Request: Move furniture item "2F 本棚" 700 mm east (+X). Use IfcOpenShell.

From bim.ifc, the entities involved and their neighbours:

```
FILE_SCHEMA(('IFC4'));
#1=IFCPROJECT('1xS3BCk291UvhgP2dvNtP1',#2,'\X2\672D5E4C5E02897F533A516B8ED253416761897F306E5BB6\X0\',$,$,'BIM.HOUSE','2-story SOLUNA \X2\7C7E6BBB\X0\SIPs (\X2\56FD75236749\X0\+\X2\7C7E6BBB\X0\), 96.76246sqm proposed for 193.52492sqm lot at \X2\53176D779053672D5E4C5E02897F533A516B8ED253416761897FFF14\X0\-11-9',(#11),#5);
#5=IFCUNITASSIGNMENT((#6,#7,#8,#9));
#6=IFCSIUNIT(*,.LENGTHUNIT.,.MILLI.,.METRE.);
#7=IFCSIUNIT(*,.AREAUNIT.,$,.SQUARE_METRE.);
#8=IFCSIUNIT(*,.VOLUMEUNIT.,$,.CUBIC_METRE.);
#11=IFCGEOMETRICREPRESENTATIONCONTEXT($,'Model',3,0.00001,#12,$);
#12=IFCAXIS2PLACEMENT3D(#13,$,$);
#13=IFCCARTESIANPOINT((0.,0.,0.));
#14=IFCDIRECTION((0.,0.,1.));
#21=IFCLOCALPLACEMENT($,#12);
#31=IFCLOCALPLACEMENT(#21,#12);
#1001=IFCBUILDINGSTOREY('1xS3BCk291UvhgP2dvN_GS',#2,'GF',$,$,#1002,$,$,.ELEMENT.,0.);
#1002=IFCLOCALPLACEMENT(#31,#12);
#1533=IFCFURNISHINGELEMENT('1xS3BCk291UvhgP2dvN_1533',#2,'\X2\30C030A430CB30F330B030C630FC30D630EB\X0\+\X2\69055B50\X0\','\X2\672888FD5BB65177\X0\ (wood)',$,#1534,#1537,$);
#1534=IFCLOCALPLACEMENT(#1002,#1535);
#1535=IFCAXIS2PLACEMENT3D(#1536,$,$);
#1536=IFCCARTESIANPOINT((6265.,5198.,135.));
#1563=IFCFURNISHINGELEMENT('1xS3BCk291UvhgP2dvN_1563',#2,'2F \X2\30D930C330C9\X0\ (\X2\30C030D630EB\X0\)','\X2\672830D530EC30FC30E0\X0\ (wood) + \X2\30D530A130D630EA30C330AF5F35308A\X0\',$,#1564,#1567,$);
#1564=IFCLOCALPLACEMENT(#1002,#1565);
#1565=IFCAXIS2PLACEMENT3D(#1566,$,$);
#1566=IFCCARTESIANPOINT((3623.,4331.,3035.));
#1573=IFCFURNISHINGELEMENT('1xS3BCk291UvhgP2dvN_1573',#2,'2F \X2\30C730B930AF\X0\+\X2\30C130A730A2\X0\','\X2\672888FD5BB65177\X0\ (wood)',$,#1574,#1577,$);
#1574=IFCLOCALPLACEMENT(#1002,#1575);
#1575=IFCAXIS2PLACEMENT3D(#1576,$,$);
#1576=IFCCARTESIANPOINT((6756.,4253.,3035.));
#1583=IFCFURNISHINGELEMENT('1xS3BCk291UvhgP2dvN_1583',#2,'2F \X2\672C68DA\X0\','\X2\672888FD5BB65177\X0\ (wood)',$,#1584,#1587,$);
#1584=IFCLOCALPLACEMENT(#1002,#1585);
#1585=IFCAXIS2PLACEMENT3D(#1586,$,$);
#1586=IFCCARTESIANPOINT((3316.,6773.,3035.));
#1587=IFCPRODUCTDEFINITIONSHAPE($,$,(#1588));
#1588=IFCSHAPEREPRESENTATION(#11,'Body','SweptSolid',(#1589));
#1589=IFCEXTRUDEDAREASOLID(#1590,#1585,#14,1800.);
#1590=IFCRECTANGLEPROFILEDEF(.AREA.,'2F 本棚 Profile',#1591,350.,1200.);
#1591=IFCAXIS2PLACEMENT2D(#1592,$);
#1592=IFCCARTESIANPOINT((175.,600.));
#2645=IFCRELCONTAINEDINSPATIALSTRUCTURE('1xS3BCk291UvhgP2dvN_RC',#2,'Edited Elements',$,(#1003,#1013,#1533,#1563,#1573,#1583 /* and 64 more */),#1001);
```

```python
import ifcopenshell
import ifcopenshell.api.geometry
import ifcopenshell.util.placement
import ifcopenshell.util.unit

model = ifcopenshell.open("bim.ifc")
unit_scale = ifcopenshell.util.unit.calculate_unit_scale(model)

item = model.by_id(1583)
matrix = ifcopenshell.util.placement.get_local_placement(item.ObjectPlacement)
matrix[0, 3] += 0.7 / unit_scale
ifcopenshell.api.geometry.edit_object_placement(model, product=item, matrix=matrix, is_si=False)

print(ifcopenshell.util.placement.get_local_placement(item.ObjectPlacement).round(3) + 0.0)

model.write("bim_rev.ifc")
```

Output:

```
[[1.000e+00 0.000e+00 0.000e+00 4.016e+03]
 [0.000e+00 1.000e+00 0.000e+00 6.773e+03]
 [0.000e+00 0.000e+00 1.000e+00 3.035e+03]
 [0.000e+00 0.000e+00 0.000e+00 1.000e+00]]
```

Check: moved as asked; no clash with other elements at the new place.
